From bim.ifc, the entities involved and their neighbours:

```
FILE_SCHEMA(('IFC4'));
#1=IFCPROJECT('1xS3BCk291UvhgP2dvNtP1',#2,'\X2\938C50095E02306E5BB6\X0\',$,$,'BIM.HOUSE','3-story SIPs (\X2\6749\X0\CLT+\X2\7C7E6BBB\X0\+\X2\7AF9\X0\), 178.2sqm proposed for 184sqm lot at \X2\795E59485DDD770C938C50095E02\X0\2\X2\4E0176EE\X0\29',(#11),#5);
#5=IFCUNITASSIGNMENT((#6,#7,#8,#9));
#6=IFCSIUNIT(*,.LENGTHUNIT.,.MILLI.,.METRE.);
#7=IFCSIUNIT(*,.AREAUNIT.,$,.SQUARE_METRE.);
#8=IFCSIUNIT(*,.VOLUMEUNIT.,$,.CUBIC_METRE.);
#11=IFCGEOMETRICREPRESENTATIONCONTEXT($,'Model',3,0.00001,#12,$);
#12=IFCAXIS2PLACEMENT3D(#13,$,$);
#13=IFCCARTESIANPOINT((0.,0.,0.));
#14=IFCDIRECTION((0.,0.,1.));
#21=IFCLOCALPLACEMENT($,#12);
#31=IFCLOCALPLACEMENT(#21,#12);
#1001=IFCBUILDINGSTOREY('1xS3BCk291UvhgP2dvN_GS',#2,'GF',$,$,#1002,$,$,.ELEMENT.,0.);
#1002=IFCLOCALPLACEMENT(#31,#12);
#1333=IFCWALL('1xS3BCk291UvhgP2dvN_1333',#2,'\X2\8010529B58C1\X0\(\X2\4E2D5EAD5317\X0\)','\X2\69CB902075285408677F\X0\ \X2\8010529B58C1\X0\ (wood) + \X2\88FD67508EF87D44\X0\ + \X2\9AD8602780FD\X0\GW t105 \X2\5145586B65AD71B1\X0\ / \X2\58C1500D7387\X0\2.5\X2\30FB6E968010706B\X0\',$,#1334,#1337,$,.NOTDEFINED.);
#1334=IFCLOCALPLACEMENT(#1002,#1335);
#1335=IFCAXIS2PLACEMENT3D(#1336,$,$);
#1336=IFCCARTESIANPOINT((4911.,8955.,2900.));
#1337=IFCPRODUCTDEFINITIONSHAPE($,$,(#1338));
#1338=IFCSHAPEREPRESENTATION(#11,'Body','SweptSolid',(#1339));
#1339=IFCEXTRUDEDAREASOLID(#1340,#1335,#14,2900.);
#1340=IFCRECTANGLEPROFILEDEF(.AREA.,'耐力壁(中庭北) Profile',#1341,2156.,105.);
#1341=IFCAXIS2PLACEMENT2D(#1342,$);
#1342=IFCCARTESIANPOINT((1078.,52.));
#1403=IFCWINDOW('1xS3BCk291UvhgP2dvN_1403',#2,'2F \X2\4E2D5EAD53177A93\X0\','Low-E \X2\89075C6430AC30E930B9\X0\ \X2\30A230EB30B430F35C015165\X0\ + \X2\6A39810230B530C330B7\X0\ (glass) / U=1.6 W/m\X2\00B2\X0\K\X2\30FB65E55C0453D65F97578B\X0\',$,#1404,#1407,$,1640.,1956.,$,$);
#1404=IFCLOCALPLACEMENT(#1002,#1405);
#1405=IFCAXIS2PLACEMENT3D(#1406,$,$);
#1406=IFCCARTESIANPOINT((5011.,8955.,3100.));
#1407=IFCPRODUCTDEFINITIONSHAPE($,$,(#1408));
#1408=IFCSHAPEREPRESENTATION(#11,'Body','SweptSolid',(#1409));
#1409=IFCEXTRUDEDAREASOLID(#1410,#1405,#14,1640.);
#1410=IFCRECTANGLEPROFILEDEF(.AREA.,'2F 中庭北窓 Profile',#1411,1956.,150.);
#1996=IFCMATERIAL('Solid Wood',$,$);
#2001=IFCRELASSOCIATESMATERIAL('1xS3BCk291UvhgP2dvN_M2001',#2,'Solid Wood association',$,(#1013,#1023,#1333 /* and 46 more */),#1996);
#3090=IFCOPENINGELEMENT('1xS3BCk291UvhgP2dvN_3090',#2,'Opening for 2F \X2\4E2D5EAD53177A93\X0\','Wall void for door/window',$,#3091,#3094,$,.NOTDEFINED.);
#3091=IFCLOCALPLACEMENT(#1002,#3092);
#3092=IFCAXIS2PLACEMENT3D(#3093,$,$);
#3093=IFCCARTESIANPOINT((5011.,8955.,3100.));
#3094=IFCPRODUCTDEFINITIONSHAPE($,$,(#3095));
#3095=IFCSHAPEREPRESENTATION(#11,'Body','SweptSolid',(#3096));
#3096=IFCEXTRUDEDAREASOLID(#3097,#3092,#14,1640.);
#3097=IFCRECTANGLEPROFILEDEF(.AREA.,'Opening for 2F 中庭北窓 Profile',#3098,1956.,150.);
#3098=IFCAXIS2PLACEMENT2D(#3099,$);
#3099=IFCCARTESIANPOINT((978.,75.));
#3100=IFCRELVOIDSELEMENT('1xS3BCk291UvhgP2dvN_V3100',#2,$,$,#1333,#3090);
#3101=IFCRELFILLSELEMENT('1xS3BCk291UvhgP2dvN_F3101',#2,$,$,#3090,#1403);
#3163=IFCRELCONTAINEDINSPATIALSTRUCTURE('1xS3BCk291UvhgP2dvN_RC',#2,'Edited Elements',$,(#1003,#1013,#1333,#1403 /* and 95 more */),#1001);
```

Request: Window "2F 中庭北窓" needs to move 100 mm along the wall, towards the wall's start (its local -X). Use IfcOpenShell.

```python
import ifcopenshell
import ifcopenshell.api.geometry
import ifcopenshell.util.placement
import ifcopenshell.util.unit

model = ifcopenshell.open("bim.ifc")
unit_scale = ifcopenshell.util.unit.calculate_unit_scale(model)

window = model.by_guid("1xS3BCk291UvhgP2dvN_1403")
opening = window.FillsVoids[0].RelatingOpeningElement
wall = opening.VoidsElements[0].RelatingBuildingElement

wall_matrix = ifcopenshell.util.placement.get_local_placement(wall.ObjectPlacement)
shift = wall_matrix[:3, 0] * -0.1 / unit_scale
before = ifcopenshell.util.placement.get_local_placement(window.ObjectPlacement)[:3, 3].copy()

# The window is not placed relative to its opening, so move both.
for product in (opening, window):
    matrix = ifcopenshell.util.placement.get_local_placement(product.ObjectPlacement)
    matrix[:3, 3] += shift
    ifcopenshell.api.geometry.edit_object_placement(model, product=product, matrix=matrix, is_si=False)

after = ifcopenshell.util.placement.get_local_placement(window.ObjectPlacement)[:3, 3]
print("window moved by", (after - before).round(3) + 0.0)

model.write("bim_v2.ifc")
```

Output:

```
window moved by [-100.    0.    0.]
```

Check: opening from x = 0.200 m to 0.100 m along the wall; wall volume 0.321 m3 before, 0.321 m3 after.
